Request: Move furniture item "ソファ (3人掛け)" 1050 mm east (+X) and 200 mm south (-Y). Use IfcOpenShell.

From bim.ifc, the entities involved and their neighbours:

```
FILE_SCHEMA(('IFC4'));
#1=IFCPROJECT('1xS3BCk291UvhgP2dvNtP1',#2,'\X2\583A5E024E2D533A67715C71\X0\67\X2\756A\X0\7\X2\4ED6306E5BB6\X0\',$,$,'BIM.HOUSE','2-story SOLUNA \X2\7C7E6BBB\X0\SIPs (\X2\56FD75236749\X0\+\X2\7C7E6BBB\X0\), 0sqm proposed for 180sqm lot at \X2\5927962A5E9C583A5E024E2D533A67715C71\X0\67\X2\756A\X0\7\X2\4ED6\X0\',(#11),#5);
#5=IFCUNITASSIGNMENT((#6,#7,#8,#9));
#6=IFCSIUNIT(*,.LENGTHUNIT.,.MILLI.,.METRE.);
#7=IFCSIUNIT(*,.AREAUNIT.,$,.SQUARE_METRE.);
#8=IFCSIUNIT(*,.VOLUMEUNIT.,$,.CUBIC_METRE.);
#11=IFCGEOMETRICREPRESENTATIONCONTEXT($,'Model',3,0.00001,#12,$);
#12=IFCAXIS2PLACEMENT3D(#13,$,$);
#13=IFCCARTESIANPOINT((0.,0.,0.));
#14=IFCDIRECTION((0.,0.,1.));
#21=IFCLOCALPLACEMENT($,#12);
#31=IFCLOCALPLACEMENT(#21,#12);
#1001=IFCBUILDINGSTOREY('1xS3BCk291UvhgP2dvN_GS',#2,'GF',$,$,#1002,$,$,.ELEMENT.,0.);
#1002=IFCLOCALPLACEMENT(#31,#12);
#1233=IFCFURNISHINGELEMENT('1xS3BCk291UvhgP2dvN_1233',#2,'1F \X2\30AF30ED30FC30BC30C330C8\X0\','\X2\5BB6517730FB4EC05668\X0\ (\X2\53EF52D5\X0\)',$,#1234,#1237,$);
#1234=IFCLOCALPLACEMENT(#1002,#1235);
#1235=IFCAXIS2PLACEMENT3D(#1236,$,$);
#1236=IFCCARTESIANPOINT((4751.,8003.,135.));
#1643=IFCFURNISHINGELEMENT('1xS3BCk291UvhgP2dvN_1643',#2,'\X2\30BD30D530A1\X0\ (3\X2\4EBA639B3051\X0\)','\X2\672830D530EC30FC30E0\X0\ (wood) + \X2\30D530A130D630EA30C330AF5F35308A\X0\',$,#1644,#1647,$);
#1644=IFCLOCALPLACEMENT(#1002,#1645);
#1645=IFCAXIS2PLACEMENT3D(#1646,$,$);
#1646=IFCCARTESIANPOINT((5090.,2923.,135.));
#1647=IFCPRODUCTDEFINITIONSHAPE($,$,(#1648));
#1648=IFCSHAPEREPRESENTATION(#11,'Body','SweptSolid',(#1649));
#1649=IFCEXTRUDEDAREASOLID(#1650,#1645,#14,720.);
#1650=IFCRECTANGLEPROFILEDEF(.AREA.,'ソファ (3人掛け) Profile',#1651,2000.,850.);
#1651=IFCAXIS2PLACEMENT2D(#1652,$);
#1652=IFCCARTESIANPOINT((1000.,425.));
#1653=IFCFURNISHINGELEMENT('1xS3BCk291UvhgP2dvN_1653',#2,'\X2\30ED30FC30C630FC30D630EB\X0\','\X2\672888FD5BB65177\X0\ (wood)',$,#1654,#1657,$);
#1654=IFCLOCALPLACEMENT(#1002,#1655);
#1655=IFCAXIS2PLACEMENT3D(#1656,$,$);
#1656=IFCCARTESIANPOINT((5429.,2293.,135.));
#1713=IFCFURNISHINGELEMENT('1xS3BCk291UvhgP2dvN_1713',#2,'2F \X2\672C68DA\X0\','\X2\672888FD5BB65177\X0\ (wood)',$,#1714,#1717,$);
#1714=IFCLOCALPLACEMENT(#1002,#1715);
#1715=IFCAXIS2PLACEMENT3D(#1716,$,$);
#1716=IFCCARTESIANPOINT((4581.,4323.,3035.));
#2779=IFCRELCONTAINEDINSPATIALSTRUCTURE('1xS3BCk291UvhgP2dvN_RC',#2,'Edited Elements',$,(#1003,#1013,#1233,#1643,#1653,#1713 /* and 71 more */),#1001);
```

```python
import ifcopenshell
import ifcopenshell.api.geometry
import ifcopenshell.util.placement
import ifcopenshell.util.unit

model = ifcopenshell.open("bim.ifc")
unit_scale = ifcopenshell.util.unit.calculate_unit_scale(model)

item = model.by_id(1643)
matrix = ifcopenshell.util.placement.get_local_placement(item.ObjectPlacement)
matrix[0, 3] += 1.05 / unit_scale
matrix[1, 3] -= 0.2 / unit_scale
ifcopenshell.api.geometry.edit_object_placement(model, product=item, matrix=matrix, is_si=False)

print(ifcopenshell.util.placement.get_local_placement(item.ObjectPlacement).round(3) + 0.0)

model.write("bim_rev.ifc")
```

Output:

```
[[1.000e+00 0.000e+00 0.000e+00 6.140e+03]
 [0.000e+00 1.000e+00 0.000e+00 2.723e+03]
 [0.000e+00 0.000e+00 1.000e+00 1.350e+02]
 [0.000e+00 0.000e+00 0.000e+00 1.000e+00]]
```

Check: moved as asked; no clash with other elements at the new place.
